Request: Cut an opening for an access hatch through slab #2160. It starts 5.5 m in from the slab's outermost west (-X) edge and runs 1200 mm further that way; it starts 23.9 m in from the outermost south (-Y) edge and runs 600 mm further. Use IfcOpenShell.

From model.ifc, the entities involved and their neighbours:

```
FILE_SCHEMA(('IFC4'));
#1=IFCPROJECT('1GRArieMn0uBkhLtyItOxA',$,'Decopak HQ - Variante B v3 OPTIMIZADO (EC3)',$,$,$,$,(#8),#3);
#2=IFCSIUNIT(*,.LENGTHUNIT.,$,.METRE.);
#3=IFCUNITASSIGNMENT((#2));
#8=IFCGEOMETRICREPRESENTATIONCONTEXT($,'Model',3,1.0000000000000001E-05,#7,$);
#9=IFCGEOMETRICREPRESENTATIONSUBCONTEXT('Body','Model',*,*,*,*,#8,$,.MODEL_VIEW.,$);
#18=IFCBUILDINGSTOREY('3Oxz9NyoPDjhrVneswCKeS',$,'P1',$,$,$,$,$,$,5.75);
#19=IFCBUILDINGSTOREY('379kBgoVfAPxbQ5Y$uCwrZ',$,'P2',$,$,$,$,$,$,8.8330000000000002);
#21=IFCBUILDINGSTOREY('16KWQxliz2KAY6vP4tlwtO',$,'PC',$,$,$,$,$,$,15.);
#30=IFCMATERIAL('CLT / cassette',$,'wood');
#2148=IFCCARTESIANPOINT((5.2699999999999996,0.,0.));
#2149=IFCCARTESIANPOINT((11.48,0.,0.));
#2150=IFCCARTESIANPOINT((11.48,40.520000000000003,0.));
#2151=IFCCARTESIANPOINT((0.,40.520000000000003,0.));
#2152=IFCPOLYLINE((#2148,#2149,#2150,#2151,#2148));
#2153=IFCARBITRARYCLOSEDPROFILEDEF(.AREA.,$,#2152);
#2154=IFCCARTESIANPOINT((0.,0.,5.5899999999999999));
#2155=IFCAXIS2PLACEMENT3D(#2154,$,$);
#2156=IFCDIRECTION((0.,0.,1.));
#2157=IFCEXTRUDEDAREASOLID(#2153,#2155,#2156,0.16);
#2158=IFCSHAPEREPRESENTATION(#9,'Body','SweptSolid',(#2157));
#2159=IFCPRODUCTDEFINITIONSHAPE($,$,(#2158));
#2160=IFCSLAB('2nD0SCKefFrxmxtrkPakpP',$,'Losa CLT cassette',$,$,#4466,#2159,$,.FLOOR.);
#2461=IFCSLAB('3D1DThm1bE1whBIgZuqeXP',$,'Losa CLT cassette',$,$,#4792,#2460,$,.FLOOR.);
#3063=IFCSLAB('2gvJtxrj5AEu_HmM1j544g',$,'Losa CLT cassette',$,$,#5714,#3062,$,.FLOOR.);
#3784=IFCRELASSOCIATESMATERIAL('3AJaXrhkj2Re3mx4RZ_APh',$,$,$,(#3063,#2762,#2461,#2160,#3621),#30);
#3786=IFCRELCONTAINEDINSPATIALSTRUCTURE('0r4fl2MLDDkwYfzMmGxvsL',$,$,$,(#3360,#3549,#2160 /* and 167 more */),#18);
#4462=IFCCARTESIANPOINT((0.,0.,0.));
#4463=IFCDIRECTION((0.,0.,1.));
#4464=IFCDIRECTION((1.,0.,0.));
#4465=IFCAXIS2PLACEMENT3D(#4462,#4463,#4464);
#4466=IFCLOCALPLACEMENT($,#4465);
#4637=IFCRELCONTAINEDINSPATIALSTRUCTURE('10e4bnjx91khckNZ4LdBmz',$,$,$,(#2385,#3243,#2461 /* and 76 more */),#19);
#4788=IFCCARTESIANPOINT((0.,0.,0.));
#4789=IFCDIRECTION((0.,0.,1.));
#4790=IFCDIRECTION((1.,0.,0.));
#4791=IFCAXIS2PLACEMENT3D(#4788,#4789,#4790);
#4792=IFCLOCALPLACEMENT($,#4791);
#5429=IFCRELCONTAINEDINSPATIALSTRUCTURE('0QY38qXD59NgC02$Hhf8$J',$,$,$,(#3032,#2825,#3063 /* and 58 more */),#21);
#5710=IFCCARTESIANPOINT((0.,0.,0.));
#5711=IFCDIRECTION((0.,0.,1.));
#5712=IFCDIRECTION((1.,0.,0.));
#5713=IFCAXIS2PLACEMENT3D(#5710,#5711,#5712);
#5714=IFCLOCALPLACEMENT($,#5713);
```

```python
import numpy as np
import ifcopenshell
import ifcopenshell.api.feature
import ifcopenshell.api.geometry
import ifcopenshell.api.root
import ifcopenshell.geom
import ifcopenshell.util.placement
import ifcopenshell.util.representation
import ifcopenshell.util.shape
import ifcopenshell.util.unit

model = ifcopenshell.open("model.ifc")
unit_scale = ifcopenshell.util.unit.calculate_unit_scale(model)
settings = ifcopenshell.geom.settings()


def volume(element):
    """Net volume in cubic metres, openings subtracted."""
    shape = ifcopenshell.geom.create_shape(settings, element)
    return ifcopenshell.util.shape.get_volume(shape.geometry)


slab = model.by_guid("2nD0SCKefFrxmxtrkPakpP")
before = volume(slab)

# Extent in the slab's own axes, in metres. The edges named are its -X and -Y sides.
slab_shape = ifcopenshell.geom.create_shape(settings, slab)
vertices = ifcopenshell.util.shape.get_vertices(slab_shape.geometry)
x_min, y_min, bottom = vertices.min(axis=0)
top = vertices[:, 2].max()

opening = ifcopenshell.api.root.create_entity(model, ifc_class="IfcOpeningElement", name="Access hatch opening", predefined_type="OPENING")
context = ifcopenshell.util.representation.get_context(model, "Model", "Body", "MODEL_VIEW")
width, depth = 1.2, 0.6
outline = [(0.0, 0.0), (width, 0.0), (width, depth), (0.0, depth), (0.0, 0.0)]
# Overshoot both faces by 50 mm so the cut is clean.
shape = ifcopenshell.api.geometry.add_slab_representation(
    model, context=context, depth=top - bottom + 0.1, polyline=outline
)
ifcopenshell.api.geometry.assign_representation(model, product=opening, representation=shape)

matrix = ifcopenshell.util.placement.get_local_placement(slab.ObjectPlacement)
matrix[:, 3] = matrix @ np.append(np.array([x_min + 5.5, y_min + 23.9, bottom - 0.05]) / unit_scale, 1.0)
ifcopenshell.api.geometry.edit_object_placement(model, product=opening, matrix=matrix, is_si=False)
ifcopenshell.api.feature.add_feature(model, feature=opening, element=slab)

after = volume(slab)

print(f"slab volume {before:.3f} -> {after:.3f} m3")

model.write("model_updated.ifc")
```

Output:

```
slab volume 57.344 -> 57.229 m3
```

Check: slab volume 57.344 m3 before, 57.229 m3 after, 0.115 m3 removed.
